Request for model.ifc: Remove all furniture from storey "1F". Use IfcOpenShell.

First a look at what the model holds.

```python
import ifcopenshell
import ifcopenshell.util.element

model = ifcopenshell.open("model.ifc")
print(model.schema)
storey = next(s for s in model.by_type("IfcBuildingStorey") if s.Name == "1F")
furniture = [e for e in ifcopenshell.util.element.get_decomposition(storey) if e.is_a("IfcFurnishingElement")]
seen = {}
for e in furniture:
    element_type = ifcopenshell.util.element.get_type(e)
    name = element_type.Name if element_type not in (None, e) else None
    seen[name] = seen.get(name, 0) + 1
for name, count in sorted(seen.items(), key=str):
    print(count, "x", name)
```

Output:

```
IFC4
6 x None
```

```python
import ifcopenshell
import ifcopenshell.api.root
import ifcopenshell.util.element

model = ifcopenshell.open("model.ifc")

storey = next(s for s in model.by_type("IfcBuildingStorey") if s.Name == "1F")
furniture = [e for e in ifcopenshell.util.element.get_decomposition(storey) if e.is_a("IfcFurnishingElement")]

for e in furniture:
    ifcopenshell.api.root.remove_product(model, product=e)
print(len(furniture), "removed")

model.write("model_rev.ifc")
```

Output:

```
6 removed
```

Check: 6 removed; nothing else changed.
